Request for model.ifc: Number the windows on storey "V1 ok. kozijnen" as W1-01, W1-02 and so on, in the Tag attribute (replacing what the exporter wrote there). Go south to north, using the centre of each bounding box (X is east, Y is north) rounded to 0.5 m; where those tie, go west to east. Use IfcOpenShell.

First a look at what the model holds.

```python
import ifcopenshell
import ifcopenshell.util.element
import ifcopenshell.util.placement

model = ifcopenshell.open("model.ifc")
print(model.schema)
storey = next(s for s in model.by_type("IfcBuildingStorey") if s.Name == "V1 ok. kozijnen")
windows = [e for e in ifcopenshell.util.element.get_decomposition(storey) if e.is_a("IfcWindow")]
for e in sorted(windows, key=lambda e: e.id()):
    origin = ifcopenshell.util.placement.get_local_placement(e.ObjectPlacement)[:3, 3]
    print(e.id(), e.Tag, e.Name, origin.round(2) + 0.0, sep=" | ")
```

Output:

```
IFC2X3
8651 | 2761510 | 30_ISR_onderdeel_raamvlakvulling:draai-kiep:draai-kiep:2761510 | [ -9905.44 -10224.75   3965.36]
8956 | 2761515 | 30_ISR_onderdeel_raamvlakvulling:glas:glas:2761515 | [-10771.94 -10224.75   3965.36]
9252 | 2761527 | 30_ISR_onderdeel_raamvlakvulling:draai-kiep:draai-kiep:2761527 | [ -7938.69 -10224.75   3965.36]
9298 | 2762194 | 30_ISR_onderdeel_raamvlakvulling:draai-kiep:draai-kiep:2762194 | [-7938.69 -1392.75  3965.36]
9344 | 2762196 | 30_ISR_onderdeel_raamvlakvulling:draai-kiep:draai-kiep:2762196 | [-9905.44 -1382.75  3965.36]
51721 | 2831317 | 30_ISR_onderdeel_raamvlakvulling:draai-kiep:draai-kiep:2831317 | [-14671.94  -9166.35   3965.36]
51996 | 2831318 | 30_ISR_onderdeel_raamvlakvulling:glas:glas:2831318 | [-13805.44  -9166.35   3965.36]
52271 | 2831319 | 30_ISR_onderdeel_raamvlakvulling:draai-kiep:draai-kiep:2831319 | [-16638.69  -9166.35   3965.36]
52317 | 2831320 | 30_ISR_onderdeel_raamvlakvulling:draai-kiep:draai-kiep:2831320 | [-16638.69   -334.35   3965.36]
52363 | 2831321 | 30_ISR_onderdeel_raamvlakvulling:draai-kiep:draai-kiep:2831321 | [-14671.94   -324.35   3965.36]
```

```python
import ifcopenshell
import ifcopenshell.geom
import ifcopenshell.util.element
import ifcopenshell.util.shape

model = ifcopenshell.open("model.ifc")
settings = ifcopenshell.geom.settings()
settings.set("use-world-coords", True)


def centre(element):
    shape = ifcopenshell.geom.create_shape(settings, element)
    return ifcopenshell.util.shape.get_bbox_centroid(shape.geometry)


storey = next(s for s in model.by_type("IfcBuildingStorey") if s.Name == "V1 ok. kozijnen")
windows = [e for e in ifcopenshell.util.element.get_decomposition(storey) if e.is_a("IfcWindow")]

# Insertion points can sit at a corner or the storey origin, so sort by the geometry (in metres).
centres = {e: centre(e) for e in windows}
windows.sort(key=lambda e: (round(centres[e][1] / 0.5), centres[e][0]))

for i, e in enumerate(windows, start=1):
    number = f"W1-{i:02d}"
    e.Tag = number
    print(e.id(), number)

model.write("model_rev.ifc")
```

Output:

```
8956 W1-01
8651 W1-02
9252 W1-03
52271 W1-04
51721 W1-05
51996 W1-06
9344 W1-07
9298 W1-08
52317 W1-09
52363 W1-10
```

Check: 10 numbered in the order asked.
